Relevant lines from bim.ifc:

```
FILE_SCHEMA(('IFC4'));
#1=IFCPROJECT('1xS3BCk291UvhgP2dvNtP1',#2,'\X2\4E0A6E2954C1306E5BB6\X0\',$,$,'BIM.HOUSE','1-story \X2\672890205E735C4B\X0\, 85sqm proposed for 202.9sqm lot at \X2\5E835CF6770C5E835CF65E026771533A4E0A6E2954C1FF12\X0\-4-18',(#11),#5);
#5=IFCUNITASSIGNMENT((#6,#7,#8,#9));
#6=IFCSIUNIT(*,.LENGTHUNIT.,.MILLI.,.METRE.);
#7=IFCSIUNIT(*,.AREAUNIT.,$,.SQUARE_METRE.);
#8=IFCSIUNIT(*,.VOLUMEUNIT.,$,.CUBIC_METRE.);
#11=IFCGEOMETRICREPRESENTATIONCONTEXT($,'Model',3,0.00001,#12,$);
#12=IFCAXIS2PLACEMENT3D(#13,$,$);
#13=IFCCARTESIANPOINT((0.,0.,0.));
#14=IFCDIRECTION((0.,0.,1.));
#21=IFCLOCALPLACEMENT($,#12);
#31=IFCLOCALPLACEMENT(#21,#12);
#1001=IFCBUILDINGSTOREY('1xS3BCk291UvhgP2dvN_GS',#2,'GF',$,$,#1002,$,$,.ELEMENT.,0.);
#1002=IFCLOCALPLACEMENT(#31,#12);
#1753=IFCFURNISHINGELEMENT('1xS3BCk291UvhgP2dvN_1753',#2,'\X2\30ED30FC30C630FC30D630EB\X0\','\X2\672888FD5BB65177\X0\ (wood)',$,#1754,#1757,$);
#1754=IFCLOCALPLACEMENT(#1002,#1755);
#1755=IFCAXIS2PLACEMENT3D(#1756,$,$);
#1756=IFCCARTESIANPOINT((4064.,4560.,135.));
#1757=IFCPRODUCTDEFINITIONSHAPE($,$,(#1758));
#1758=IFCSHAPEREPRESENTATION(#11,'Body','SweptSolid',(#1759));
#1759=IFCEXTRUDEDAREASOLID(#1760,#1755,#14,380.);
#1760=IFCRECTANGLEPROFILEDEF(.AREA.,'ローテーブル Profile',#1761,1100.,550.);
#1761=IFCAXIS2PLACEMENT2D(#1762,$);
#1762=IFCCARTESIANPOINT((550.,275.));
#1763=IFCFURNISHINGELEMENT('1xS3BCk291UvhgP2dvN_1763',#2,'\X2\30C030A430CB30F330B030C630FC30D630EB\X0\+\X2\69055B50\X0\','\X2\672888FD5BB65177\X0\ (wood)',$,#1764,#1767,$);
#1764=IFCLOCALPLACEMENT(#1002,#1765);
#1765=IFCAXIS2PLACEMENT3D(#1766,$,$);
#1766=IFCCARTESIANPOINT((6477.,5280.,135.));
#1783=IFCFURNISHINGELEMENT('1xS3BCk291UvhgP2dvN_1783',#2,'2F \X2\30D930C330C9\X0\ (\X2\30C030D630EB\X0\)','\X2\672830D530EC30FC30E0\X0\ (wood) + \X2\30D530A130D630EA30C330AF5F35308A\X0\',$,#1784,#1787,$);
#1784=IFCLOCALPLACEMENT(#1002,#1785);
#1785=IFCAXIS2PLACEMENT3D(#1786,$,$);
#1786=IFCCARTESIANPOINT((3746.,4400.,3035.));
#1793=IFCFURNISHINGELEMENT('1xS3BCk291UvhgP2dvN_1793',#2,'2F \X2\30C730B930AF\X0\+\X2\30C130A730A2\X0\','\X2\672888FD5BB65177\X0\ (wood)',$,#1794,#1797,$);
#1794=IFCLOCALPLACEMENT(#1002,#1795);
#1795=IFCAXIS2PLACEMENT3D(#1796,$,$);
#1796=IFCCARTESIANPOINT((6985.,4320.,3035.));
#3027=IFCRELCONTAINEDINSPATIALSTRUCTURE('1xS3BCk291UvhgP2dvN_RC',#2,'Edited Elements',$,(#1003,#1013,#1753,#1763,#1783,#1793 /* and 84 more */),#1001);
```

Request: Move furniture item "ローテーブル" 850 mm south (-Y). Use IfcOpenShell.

```python
import ifcopenshell
import ifcopenshell.api.geometry
import ifcopenshell.util.placement
import ifcopenshell.util.unit

model = ifcopenshell.open("bim.ifc")
unit_scale = ifcopenshell.util.unit.calculate_unit_scale(model)

item = model.by_guid("1xS3BCk291UvhgP2dvN_1753")
matrix = ifcopenshell.util.placement.get_local_placement(item.ObjectPlacement)
matrix[1, 3] -= 0.85 / unit_scale
ifcopenshell.api.geometry.edit_object_placement(model, product=item, matrix=matrix, is_si=False)

print(ifcopenshell.util.placement.get_local_placement(item.ObjectPlacement).round(3) + 0.0)

model.write("bim-out.ifc")
```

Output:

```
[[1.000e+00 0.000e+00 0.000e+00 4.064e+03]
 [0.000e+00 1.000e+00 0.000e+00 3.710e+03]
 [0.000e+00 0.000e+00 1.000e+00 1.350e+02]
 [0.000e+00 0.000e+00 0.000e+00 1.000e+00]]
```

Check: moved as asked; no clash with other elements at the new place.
